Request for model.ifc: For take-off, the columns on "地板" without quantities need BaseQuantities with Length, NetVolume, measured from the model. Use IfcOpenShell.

First a look at what the model holds.

```python
import ifcopenshell
import ifcopenshell.util.element
import ifcopenshell.util.unit

model = ifcopenshell.open("model.ifc")
print(model.schema)
for unit_type in ("LENGTHUNIT", "AREAUNIT", "VOLUMEUNIT"):
    print(unit_type, ifcopenshell.util.unit.calculate_unit_scale(model, unit_type))
storey = next(s for s in model.by_type("IfcBuildingStorey") if s.Name == "地板")
columns = [e for e in ifcopenshell.util.element.get_decomposition(storey) if e.is_a("IfcColumn")]
for e in sorted(columns, key=lambda e: e.id()):
    print(e.id(), e.is_a(), e.Name, list(ifcopenshell.util.element.get_psets(e, qtos_only=True)), sep=" | ")
```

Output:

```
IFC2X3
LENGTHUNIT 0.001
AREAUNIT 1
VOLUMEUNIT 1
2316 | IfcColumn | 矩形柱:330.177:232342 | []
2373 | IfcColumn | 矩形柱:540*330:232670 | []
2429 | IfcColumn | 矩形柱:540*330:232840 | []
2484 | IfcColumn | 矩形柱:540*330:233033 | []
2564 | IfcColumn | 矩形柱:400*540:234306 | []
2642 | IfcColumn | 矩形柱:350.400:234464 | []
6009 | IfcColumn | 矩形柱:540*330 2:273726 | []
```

```python
import ifcopenshell
import ifcopenshell.api.pset
import ifcopenshell.geom
import ifcopenshell.util.element
import ifcopenshell.util.shape
import ifcopenshell.util.unit

model = ifcopenshell.open("model.ifc")
unit_scale = ifcopenshell.util.unit.calculate_unit_scale(model)
volume_scale = ifcopenshell.util.unit.calculate_unit_scale(model, "VOLUMEUNIT")
settings = ifcopenshell.geom.settings()

storey = next(s for s in model.by_type("IfcBuildingStorey") if s.Name == "地板")
columns = [e for e in ifcopenshell.util.element.get_decomposition(storey) if e.is_a("IfcColumn")]

for e in sorted(columns, key=lambda e: e.id()):
    if ifcopenshell.util.element.get_psets(e, qtos_only=True, should_inherit=False):
        continue
    # Geometry comes back in metres, in the element's own axes.
    shape = ifcopenshell.geom.create_shape(settings, e)
    values = {
        "Length": ifcopenshell.util.shape.get_z(shape.geometry) / unit_scale,
        "NetVolume": ifcopenshell.util.shape.get_volume(shape.geometry) / volume_scale,
    }
    qto = ifcopenshell.api.pset.add_qto(model, product=e, name="BaseQuantities")
    ifcopenshell.api.pset.edit_qto(model, qto=qto, properties=values)
    print(e.id(), {k: round(v, 3) for k, v in values.items()})

model.write("model_updated.ifc")
```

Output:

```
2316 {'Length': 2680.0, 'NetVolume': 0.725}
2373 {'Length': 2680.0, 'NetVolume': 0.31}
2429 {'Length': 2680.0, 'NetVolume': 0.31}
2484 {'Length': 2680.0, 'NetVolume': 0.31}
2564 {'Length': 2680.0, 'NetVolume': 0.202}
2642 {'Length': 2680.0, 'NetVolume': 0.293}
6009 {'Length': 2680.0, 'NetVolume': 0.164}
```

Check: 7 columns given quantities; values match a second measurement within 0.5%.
